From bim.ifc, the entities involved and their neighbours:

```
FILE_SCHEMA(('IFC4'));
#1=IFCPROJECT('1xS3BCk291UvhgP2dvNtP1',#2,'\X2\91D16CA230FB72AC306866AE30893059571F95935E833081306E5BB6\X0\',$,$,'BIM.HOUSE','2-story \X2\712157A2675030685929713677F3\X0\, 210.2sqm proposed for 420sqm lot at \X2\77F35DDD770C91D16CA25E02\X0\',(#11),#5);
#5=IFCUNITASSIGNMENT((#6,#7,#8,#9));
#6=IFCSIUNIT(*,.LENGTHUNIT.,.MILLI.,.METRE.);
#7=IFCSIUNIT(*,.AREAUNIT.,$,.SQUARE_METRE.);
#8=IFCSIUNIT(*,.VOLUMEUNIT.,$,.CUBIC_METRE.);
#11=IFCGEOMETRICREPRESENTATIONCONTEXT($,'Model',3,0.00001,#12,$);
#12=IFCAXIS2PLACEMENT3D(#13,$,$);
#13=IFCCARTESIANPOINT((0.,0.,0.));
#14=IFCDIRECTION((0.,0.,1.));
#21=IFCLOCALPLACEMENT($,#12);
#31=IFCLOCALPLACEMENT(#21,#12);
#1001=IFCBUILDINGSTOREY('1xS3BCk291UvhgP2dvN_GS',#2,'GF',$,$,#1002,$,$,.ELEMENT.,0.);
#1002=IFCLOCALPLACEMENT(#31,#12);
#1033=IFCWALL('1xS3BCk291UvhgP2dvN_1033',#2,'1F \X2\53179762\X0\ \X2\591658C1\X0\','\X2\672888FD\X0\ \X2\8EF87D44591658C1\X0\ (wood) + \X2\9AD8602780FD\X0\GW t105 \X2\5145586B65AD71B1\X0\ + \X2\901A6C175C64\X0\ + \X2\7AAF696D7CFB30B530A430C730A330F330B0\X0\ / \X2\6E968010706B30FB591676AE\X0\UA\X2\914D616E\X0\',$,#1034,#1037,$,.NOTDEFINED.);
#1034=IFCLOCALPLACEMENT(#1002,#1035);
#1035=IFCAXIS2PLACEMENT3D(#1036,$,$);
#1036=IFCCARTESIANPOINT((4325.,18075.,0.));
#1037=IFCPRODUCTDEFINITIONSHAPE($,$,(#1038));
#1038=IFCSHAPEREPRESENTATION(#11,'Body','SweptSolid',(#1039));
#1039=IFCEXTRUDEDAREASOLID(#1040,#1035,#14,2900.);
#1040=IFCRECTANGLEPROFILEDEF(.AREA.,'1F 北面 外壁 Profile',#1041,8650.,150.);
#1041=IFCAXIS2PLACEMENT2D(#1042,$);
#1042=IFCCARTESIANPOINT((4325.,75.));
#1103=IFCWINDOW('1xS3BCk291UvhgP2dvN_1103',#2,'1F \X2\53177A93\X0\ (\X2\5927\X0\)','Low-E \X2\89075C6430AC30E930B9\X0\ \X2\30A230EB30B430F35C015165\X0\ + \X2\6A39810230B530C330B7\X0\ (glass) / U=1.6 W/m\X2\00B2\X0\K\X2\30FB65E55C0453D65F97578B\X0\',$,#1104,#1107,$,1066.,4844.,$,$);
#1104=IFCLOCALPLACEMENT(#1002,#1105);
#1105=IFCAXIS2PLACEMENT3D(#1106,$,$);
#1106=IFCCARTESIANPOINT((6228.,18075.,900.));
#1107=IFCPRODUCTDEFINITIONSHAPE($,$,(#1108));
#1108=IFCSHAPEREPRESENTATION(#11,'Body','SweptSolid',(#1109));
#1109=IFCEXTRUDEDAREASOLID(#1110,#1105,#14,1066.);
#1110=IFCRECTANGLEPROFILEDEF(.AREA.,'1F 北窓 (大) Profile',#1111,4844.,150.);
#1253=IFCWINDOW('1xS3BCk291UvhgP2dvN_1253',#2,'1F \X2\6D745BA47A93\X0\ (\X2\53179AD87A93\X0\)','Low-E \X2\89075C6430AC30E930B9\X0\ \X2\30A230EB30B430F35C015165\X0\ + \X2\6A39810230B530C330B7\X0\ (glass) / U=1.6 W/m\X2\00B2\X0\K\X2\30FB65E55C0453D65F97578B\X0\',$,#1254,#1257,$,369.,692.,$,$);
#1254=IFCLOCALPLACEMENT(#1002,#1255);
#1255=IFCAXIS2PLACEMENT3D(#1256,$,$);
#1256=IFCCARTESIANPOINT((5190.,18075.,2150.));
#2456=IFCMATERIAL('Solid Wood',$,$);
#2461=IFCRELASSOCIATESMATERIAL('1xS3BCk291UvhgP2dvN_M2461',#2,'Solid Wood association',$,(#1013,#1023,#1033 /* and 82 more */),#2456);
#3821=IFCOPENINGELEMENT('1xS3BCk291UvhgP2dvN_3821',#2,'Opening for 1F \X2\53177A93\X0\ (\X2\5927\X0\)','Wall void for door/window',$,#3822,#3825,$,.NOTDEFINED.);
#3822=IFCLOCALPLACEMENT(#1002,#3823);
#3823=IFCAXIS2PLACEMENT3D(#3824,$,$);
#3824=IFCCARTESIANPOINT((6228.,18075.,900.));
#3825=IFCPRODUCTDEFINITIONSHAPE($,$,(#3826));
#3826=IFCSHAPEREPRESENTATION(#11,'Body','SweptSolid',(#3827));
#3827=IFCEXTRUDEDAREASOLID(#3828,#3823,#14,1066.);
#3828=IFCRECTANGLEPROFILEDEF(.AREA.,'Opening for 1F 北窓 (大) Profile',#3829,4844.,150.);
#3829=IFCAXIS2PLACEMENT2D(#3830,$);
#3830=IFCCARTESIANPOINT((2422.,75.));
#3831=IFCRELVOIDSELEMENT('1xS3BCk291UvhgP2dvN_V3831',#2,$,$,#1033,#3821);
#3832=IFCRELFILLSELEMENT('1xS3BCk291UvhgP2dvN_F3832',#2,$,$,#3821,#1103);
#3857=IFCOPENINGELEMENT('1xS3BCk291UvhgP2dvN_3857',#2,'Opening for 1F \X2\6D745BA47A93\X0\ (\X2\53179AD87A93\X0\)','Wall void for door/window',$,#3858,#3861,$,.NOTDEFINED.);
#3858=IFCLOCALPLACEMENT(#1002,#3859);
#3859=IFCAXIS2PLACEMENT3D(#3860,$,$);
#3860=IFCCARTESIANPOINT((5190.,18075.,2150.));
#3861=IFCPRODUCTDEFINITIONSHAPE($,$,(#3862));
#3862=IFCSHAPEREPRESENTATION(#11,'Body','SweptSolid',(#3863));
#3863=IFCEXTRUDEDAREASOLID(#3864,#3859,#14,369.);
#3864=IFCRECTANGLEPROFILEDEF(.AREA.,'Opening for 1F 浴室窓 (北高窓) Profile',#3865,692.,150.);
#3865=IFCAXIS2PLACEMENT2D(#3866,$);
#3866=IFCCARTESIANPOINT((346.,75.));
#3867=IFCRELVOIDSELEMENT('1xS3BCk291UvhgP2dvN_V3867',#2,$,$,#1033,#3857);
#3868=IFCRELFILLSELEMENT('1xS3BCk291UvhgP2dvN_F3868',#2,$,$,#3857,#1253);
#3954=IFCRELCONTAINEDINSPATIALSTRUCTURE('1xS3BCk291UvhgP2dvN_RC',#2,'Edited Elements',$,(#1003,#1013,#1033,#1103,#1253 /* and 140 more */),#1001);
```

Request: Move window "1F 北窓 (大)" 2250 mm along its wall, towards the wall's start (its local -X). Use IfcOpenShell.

```python
import ifcopenshell
import ifcopenshell.api.geometry
import ifcopenshell.util.placement
import ifcopenshell.util.unit

model = ifcopenshell.open("bim.ifc")
unit_scale = ifcopenshell.util.unit.calculate_unit_scale(model)

window = model.by_guid("1xS3BCk291UvhgP2dvN_1103")
opening = window.FillsVoids[0].RelatingOpeningElement
wall = opening.VoidsElements[0].RelatingBuildingElement

wall_matrix = ifcopenshell.util.placement.get_local_placement(wall.ObjectPlacement)
shift = wall_matrix[:3, 0] * -2.25 / unit_scale
before = ifcopenshell.util.placement.get_local_placement(window.ObjectPlacement)[:3, 3].copy()

# The window is not placed relative to its opening, so move both.
for product in (opening, window):
    matrix = ifcopenshell.util.placement.get_local_placement(product.ObjectPlacement)
    matrix[:3, 3] += shift
    ifcopenshell.api.geometry.edit_object_placement(model, product=product, matrix=matrix, is_si=False)

after = ifcopenshell.util.placement.get_local_placement(window.ObjectPlacement)[:3, 3]
print("window moved by", (after - before).round(3) + 0.0)

model.write("bim_v2.ifc")
```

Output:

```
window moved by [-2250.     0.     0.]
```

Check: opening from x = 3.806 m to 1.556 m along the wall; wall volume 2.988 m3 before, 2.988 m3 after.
